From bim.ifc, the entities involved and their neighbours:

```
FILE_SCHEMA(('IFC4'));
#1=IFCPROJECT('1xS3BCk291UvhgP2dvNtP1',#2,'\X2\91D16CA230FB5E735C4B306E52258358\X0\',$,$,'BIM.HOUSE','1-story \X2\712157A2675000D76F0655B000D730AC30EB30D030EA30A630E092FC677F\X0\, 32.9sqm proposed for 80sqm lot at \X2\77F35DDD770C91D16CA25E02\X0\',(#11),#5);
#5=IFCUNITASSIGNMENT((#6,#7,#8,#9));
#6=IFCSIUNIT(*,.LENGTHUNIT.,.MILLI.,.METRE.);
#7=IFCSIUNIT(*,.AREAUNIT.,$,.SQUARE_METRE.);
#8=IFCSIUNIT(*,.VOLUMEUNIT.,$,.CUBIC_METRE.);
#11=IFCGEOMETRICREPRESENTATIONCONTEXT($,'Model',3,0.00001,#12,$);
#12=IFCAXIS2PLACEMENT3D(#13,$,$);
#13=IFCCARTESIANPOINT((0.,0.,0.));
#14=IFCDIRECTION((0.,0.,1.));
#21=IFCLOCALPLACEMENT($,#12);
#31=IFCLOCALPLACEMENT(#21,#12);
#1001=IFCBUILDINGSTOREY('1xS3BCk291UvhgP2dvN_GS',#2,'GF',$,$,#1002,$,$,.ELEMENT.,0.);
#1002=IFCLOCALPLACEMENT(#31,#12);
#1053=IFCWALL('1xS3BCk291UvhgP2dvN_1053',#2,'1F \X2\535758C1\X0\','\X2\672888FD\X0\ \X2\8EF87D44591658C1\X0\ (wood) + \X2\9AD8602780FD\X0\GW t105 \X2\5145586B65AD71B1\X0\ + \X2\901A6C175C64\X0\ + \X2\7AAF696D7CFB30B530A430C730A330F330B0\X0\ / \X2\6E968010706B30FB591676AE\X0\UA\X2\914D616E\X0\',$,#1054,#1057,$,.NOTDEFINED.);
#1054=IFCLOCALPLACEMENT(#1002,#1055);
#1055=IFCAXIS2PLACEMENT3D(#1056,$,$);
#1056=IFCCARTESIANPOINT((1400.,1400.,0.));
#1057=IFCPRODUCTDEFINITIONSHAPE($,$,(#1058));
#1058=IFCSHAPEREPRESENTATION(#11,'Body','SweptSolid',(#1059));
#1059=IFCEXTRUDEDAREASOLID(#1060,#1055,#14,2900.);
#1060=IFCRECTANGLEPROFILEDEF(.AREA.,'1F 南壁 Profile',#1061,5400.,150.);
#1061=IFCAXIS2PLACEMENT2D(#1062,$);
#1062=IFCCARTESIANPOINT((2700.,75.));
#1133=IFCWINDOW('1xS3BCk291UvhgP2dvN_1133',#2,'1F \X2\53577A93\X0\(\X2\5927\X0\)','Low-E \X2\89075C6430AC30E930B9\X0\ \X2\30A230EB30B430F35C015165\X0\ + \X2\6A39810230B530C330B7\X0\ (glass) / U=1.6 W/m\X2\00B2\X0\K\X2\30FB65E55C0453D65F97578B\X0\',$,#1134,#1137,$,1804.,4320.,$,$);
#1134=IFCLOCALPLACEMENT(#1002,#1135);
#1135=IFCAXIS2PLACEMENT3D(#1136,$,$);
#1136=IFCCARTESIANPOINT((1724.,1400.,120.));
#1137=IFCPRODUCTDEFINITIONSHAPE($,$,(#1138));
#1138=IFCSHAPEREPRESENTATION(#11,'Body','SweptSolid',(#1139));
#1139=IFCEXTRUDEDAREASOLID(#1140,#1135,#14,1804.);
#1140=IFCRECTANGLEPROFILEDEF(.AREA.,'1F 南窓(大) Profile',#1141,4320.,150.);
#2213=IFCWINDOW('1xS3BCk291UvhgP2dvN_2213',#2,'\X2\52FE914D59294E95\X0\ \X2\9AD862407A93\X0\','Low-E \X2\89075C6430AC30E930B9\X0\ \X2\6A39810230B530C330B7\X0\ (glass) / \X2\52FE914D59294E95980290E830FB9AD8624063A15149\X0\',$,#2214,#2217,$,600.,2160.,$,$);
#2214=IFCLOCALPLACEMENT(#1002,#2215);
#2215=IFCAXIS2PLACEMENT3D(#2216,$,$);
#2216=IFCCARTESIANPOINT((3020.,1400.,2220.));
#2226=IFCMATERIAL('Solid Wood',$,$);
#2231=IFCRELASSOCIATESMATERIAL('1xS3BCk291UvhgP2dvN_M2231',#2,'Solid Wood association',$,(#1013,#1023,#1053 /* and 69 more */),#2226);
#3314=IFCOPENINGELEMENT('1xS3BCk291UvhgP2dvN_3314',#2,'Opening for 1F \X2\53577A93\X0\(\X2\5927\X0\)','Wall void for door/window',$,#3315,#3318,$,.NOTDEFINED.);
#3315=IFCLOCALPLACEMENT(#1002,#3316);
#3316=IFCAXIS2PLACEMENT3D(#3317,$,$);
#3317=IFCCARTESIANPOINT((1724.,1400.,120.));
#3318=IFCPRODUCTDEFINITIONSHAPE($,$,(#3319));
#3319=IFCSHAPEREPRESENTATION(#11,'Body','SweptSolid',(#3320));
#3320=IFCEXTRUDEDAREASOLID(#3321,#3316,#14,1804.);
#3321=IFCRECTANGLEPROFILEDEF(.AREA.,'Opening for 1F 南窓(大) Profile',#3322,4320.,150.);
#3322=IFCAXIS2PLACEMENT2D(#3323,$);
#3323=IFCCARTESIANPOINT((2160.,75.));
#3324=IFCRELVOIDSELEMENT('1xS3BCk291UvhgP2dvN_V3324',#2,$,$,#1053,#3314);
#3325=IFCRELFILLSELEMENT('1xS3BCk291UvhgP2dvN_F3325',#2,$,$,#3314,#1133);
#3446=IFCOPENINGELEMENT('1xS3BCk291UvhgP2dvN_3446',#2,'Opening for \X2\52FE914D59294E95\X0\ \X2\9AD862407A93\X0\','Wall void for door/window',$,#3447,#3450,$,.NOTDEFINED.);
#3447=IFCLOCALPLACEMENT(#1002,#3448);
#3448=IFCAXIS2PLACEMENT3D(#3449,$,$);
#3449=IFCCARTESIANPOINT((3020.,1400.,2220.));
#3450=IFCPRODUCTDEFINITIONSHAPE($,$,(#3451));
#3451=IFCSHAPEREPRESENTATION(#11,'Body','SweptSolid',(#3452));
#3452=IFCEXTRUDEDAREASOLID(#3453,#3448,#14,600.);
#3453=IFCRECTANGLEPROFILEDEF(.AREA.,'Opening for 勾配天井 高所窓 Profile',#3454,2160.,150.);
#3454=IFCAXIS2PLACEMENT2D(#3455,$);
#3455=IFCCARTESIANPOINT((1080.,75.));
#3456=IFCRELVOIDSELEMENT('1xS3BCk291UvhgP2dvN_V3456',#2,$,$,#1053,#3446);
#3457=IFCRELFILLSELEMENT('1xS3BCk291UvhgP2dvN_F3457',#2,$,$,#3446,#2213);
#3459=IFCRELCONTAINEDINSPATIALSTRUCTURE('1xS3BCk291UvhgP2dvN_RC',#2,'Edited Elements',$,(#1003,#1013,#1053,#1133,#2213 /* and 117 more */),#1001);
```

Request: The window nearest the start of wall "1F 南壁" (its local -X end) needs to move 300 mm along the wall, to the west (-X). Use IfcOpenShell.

```python
import ifcopenshell
import ifcopenshell.api.geometry
import ifcopenshell.util.placement
import ifcopenshell.util.unit

model = ifcopenshell.open("bim.ifc")
unit_scale = ifcopenshell.util.unit.calculate_unit_scale(model)

window = model.by_guid("1xS3BCk291UvhgP2dvN_1133")
opening = window.FillsVoids[0].RelatingOpeningElement
wall = opening.VoidsElements[0].RelatingBuildingElement

wall_matrix = ifcopenshell.util.placement.get_local_placement(wall.ObjectPlacement)
shift = wall_matrix[:3, 0] * -0.3 / unit_scale
before = ifcopenshell.util.placement.get_local_placement(window.ObjectPlacement)[:3, 3].copy()

# The window is not placed relative to its opening, so move both.
for product in (opening, window):
    matrix = ifcopenshell.util.placement.get_local_placement(product.ObjectPlacement)
    matrix[:3, 3] += shift
    ifcopenshell.api.geometry.edit_object_placement(model, product=product, matrix=matrix, is_si=False)

after = ifcopenshell.util.placement.get_local_placement(window.ObjectPlacement)[:3, 3]
print("window moved by", (after - before).round(3) + 0.0)

model.write("bim_updated.ifc")
```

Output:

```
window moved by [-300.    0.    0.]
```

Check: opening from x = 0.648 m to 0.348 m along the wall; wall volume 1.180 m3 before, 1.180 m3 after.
